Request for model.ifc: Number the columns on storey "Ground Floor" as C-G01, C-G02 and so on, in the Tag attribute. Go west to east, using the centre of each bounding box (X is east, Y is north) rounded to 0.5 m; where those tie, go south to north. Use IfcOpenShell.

First a look at what the model holds.

```python
import ifcopenshell
import ifcopenshell.util.element
import ifcopenshell.util.placement

model = ifcopenshell.open("model.ifc")
print(model.schema)
storey = next(s for s in model.by_type("IfcBuildingStorey") if s.Name == "Ground Floor")
columns = [e for e in ifcopenshell.util.element.get_decomposition(storey) if e.is_a("IfcColumn")]
for e in sorted(columns, key=lambda e: e.id()):
    origin = ifcopenshell.util.placement.get_local_placement(e.ObjectPlacement)[:3, 3]
    print(e.id(), e.Tag, e.Name, origin.round(2) + 0.0, sep=" | ")
```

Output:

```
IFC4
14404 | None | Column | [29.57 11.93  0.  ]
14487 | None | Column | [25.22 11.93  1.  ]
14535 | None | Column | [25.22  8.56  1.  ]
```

```python
import ifcopenshell
import ifcopenshell.geom
import ifcopenshell.util.element
import ifcopenshell.util.shape

model = ifcopenshell.open("model.ifc")
settings = ifcopenshell.geom.settings()
settings.set("use-world-coords", True)


def centre(element):
    shape = ifcopenshell.geom.create_shape(settings, element)
    return ifcopenshell.util.shape.get_bbox_centroid(shape.geometry)


storey = next(s for s in model.by_type("IfcBuildingStorey") if s.Name == "Ground Floor")
columns = [e for e in ifcopenshell.util.element.get_decomposition(storey) if e.is_a("IfcColumn")]

# Insertion points can sit at a corner or the storey origin, so sort by the geometry (in metres).
centres = {e: centre(e) for e in columns}
columns.sort(key=lambda e: (round(centres[e][0] / 0.5), centres[e][1]))

for i, e in enumerate(columns, start=1):
    number = f"C-G{i:02d}"
    e.Tag = number
    print(e.id(), number)

model.write("model_v2.ifc")
```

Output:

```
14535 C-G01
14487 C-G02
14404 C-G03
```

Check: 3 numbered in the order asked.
